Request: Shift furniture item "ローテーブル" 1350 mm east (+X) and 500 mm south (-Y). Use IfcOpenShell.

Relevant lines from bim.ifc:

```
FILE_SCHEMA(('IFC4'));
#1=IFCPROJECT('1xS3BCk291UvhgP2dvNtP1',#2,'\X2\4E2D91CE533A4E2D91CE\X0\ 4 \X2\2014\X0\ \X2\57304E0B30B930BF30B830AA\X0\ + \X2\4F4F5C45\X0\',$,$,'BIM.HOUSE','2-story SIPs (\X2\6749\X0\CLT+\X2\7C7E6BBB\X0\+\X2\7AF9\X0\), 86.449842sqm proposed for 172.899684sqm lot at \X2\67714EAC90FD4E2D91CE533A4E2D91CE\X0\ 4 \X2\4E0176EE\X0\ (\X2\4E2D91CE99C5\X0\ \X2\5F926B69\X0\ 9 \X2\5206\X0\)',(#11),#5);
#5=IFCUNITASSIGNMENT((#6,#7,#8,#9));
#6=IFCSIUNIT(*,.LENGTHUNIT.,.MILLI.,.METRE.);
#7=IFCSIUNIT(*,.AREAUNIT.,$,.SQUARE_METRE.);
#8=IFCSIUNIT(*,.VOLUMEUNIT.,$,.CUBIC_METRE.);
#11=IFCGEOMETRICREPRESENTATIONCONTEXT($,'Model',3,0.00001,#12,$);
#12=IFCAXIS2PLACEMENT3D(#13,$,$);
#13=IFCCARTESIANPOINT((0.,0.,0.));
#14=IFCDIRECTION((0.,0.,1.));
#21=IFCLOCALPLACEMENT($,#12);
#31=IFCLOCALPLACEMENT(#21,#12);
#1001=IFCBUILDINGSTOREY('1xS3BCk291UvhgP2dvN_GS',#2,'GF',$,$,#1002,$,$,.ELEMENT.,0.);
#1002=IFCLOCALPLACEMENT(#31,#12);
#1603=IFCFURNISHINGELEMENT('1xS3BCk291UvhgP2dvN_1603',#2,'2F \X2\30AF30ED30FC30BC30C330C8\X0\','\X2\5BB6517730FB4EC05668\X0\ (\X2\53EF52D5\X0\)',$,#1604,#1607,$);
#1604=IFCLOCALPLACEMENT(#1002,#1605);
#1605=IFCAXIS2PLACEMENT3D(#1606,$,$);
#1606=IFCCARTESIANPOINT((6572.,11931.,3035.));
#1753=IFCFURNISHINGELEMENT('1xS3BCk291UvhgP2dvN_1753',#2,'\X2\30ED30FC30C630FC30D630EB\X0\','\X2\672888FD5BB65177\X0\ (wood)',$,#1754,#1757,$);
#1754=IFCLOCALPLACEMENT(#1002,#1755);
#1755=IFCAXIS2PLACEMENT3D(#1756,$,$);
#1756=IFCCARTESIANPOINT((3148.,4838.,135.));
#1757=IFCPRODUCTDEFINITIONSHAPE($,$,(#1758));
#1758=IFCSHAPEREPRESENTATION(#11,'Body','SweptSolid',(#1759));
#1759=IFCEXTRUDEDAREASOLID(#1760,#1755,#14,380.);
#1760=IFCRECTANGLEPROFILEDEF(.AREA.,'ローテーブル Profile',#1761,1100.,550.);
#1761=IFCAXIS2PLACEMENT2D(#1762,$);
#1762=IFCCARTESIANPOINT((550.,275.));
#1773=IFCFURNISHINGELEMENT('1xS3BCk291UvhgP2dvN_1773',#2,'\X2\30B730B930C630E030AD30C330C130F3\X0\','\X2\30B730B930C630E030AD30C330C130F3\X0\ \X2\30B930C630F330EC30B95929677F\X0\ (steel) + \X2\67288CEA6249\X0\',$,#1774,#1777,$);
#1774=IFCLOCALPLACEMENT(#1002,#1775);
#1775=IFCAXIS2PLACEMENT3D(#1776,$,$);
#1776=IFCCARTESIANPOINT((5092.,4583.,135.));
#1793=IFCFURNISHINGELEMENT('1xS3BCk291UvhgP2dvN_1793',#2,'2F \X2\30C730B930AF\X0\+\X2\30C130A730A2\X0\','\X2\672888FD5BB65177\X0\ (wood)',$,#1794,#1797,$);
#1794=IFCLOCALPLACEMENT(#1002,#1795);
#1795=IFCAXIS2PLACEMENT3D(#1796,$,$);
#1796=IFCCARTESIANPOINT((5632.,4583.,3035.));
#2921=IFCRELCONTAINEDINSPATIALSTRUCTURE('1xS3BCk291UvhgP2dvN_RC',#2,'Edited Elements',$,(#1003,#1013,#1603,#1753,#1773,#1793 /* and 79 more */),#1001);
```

```python
import ifcopenshell
import ifcopenshell.api.geometry
import ifcopenshell.util.placement

model = ifcopenshell.open("bim.ifc")

item = model.by_guid("1xS3BCk291UvhgP2dvN_1753")
matrix = ifcopenshell.util.placement.get_local_placement(item.ObjectPlacement)
matrix[0, 3] += 1350.0
matrix[1, 3] -= 500.0
ifcopenshell.api.geometry.edit_object_placement(model, product=item, matrix=matrix, is_si=False)

print(ifcopenshell.util.placement.get_local_placement(item.ObjectPlacement).round(3) + 0.0)

model.write("bim_rev.ifc")
```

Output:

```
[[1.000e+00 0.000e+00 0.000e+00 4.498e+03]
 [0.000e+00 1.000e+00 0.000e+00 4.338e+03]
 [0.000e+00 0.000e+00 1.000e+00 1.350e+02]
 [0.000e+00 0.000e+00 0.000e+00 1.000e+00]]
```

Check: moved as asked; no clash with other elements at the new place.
